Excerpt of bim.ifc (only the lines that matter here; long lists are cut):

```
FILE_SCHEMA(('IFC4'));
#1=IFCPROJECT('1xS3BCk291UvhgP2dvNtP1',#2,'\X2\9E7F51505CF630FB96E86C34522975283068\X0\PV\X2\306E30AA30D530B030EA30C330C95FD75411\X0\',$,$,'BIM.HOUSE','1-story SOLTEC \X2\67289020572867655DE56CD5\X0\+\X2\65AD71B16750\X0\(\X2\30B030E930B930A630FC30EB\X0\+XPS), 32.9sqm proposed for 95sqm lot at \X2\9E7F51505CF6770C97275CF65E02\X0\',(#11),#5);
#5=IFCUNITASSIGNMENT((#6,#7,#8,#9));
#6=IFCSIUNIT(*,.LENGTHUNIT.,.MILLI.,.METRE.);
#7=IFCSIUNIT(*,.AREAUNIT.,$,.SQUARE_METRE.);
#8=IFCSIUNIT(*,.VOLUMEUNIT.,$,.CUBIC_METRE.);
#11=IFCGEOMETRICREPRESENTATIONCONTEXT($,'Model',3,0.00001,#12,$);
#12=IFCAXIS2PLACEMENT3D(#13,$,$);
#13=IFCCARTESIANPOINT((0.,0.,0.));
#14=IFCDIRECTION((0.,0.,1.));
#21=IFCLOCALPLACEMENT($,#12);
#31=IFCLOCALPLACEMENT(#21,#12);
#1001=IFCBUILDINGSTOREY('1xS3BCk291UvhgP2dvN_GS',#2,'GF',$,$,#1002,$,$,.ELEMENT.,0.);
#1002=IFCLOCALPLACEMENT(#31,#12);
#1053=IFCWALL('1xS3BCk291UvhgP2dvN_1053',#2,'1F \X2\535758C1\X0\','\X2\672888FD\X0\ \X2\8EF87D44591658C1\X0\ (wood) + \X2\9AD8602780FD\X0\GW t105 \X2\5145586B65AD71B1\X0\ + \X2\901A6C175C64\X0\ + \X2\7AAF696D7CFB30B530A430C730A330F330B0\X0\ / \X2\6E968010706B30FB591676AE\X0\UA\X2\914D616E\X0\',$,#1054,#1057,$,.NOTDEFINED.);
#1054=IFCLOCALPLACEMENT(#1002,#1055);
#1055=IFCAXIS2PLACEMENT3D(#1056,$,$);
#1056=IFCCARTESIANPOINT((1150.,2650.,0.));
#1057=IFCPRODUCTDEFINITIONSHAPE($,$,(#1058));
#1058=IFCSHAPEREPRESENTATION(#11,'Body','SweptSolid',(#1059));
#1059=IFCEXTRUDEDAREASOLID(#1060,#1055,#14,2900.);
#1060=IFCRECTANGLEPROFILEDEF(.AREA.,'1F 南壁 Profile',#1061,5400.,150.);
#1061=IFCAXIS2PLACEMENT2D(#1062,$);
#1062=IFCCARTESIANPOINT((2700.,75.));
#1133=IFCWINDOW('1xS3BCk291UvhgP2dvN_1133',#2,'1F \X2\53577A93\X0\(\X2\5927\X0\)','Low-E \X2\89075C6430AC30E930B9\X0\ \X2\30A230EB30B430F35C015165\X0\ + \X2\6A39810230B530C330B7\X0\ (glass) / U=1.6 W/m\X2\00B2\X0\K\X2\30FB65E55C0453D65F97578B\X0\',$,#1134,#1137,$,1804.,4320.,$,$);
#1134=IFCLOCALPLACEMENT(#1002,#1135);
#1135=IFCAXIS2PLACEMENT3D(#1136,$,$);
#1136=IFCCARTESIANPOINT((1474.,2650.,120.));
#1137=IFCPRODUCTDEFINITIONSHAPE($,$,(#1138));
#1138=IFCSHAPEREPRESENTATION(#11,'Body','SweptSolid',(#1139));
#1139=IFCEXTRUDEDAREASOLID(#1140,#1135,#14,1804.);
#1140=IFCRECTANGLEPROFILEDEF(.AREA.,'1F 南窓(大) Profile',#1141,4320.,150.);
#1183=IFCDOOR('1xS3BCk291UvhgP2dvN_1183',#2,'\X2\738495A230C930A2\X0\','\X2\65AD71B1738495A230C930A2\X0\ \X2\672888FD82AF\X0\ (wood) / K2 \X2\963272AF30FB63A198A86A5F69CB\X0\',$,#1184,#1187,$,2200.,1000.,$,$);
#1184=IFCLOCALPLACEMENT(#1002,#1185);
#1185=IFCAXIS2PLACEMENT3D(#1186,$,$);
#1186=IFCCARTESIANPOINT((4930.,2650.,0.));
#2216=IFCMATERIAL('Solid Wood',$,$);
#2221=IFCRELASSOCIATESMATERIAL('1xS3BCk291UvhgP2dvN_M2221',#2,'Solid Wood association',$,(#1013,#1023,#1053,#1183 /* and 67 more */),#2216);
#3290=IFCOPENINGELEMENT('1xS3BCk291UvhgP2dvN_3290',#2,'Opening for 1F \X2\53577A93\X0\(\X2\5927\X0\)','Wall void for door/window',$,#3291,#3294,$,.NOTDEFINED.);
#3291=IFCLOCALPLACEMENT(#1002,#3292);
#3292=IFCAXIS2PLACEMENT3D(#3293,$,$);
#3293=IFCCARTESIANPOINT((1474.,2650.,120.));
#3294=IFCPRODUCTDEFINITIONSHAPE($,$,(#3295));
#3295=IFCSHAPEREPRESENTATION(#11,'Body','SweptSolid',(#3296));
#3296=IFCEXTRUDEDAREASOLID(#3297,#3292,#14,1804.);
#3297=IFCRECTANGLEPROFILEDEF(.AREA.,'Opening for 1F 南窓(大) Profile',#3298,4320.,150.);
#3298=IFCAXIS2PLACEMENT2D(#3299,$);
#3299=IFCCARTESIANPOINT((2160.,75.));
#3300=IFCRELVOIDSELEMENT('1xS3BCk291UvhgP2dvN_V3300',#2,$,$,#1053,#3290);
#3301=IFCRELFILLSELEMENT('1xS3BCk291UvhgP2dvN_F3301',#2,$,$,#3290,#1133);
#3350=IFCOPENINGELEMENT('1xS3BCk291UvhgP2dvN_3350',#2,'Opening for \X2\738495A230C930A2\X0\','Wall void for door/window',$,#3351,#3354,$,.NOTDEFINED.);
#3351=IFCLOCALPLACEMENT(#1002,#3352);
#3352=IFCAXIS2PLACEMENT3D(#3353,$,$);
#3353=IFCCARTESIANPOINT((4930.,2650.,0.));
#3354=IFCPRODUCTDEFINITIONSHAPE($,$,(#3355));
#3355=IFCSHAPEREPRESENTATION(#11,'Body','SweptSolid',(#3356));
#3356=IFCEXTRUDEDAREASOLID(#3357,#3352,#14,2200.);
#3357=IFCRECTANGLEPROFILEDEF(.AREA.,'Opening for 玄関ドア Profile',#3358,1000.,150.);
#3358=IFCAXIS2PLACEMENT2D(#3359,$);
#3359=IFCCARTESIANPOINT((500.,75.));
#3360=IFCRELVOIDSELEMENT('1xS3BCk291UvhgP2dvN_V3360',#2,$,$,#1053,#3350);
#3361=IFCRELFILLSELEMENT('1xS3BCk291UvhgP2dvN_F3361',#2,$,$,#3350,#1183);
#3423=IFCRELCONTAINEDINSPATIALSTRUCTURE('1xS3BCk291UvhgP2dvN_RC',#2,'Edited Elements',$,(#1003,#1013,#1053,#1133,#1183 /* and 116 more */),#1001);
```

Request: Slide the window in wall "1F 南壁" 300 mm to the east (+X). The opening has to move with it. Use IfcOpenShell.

```python
import ifcopenshell
import ifcopenshell.api.geometry
import ifcopenshell.util.placement

model = ifcopenshell.open("bim.ifc")

window = model.by_guid("1xS3BCk291UvhgP2dvN_1133")
opening = window.FillsVoids[0].RelatingOpeningElement
wall = opening.VoidsElements[0].RelatingBuildingElement

wall_matrix = ifcopenshell.util.placement.get_local_placement(wall.ObjectPlacement)
shift = wall_matrix[:3, 0] * 300.0
before = ifcopenshell.util.placement.get_local_placement(window.ObjectPlacement)[:3, 3].copy()

# The window is not placed relative to its opening, so move both.
for product in (opening, window):
    matrix = ifcopenshell.util.placement.get_local_placement(product.ObjectPlacement)
    matrix[:3, 3] += shift
    ifcopenshell.api.geometry.edit_object_placement(model, product=product, matrix=matrix, is_si=False)

after = ifcopenshell.util.placement.get_local_placement(window.ObjectPlacement)[:3, 3]
print("window moved by", (after - before).round(3) + 0.0)

model.write("bim_rev.ifc")
```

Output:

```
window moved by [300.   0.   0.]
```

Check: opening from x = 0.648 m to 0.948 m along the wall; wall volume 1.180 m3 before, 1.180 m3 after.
